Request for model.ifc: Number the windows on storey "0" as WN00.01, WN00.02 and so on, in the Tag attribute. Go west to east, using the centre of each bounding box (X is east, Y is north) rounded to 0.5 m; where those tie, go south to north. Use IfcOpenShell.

First a look at what the model holds.

```python
import ifcopenshell
import ifcopenshell.util.element
import ifcopenshell.util.placement

model = ifcopenshell.open("model.ifc")
print(model.schema)
storey = next(s for s in model.by_type("IfcBuildingStorey") if s.Name == "0")
windows = [e for e in ifcopenshell.util.element.get_decomposition(storey) if e.is_a("IfcWindow")]
for e in sorted(windows, key=lambda e: e.id()):
    origin = ifcopenshell.util.placement.get_local_placement(e.ObjectPlacement)[:3, 3]
    print(e.id(), e.Tag, e.Name, origin.round(2) + 0.0, sep=" | ")
```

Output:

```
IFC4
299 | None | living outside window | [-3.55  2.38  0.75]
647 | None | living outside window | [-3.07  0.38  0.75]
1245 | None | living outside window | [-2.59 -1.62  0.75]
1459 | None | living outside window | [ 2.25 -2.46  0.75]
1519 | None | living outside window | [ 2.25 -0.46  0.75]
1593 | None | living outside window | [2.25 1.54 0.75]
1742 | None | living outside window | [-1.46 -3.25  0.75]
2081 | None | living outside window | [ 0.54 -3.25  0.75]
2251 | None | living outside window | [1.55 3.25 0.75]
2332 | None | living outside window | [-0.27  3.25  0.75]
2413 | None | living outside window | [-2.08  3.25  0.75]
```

```python
import ifcopenshell
import ifcopenshell.geom
import ifcopenshell.util.element
import ifcopenshell.util.shape

model = ifcopenshell.open("model.ifc")
settings = ifcopenshell.geom.settings()
settings.set("use-world-coords", True)


def centre(element):
    shape = ifcopenshell.geom.create_shape(settings, element)
    return ifcopenshell.util.shape.get_bbox_centroid(shape.geometry)


storey = next(s for s in model.by_type("IfcBuildingStorey") if s.Name == "0")
windows = [e for e in ifcopenshell.util.element.get_decomposition(storey) if e.is_a("IfcWindow")]

# Insertion points can sit at a corner or the storey origin, so sort by the geometry (in metres).
centres = {e: centre(e) for e in windows}
windows.sort(key=lambda e: (round(centres[e][0] / 0.5), centres[e][1]))

for i, e in enumerate(windows, start=1):
    number = f"WN00.{i:02d}"
    e.Tag = number
    print(e.id(), number)

model.write("model_v2.ifc")
```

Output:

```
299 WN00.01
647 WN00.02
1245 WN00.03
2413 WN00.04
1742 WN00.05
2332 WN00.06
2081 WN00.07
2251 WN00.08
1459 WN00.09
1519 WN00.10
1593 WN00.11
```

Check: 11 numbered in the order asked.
